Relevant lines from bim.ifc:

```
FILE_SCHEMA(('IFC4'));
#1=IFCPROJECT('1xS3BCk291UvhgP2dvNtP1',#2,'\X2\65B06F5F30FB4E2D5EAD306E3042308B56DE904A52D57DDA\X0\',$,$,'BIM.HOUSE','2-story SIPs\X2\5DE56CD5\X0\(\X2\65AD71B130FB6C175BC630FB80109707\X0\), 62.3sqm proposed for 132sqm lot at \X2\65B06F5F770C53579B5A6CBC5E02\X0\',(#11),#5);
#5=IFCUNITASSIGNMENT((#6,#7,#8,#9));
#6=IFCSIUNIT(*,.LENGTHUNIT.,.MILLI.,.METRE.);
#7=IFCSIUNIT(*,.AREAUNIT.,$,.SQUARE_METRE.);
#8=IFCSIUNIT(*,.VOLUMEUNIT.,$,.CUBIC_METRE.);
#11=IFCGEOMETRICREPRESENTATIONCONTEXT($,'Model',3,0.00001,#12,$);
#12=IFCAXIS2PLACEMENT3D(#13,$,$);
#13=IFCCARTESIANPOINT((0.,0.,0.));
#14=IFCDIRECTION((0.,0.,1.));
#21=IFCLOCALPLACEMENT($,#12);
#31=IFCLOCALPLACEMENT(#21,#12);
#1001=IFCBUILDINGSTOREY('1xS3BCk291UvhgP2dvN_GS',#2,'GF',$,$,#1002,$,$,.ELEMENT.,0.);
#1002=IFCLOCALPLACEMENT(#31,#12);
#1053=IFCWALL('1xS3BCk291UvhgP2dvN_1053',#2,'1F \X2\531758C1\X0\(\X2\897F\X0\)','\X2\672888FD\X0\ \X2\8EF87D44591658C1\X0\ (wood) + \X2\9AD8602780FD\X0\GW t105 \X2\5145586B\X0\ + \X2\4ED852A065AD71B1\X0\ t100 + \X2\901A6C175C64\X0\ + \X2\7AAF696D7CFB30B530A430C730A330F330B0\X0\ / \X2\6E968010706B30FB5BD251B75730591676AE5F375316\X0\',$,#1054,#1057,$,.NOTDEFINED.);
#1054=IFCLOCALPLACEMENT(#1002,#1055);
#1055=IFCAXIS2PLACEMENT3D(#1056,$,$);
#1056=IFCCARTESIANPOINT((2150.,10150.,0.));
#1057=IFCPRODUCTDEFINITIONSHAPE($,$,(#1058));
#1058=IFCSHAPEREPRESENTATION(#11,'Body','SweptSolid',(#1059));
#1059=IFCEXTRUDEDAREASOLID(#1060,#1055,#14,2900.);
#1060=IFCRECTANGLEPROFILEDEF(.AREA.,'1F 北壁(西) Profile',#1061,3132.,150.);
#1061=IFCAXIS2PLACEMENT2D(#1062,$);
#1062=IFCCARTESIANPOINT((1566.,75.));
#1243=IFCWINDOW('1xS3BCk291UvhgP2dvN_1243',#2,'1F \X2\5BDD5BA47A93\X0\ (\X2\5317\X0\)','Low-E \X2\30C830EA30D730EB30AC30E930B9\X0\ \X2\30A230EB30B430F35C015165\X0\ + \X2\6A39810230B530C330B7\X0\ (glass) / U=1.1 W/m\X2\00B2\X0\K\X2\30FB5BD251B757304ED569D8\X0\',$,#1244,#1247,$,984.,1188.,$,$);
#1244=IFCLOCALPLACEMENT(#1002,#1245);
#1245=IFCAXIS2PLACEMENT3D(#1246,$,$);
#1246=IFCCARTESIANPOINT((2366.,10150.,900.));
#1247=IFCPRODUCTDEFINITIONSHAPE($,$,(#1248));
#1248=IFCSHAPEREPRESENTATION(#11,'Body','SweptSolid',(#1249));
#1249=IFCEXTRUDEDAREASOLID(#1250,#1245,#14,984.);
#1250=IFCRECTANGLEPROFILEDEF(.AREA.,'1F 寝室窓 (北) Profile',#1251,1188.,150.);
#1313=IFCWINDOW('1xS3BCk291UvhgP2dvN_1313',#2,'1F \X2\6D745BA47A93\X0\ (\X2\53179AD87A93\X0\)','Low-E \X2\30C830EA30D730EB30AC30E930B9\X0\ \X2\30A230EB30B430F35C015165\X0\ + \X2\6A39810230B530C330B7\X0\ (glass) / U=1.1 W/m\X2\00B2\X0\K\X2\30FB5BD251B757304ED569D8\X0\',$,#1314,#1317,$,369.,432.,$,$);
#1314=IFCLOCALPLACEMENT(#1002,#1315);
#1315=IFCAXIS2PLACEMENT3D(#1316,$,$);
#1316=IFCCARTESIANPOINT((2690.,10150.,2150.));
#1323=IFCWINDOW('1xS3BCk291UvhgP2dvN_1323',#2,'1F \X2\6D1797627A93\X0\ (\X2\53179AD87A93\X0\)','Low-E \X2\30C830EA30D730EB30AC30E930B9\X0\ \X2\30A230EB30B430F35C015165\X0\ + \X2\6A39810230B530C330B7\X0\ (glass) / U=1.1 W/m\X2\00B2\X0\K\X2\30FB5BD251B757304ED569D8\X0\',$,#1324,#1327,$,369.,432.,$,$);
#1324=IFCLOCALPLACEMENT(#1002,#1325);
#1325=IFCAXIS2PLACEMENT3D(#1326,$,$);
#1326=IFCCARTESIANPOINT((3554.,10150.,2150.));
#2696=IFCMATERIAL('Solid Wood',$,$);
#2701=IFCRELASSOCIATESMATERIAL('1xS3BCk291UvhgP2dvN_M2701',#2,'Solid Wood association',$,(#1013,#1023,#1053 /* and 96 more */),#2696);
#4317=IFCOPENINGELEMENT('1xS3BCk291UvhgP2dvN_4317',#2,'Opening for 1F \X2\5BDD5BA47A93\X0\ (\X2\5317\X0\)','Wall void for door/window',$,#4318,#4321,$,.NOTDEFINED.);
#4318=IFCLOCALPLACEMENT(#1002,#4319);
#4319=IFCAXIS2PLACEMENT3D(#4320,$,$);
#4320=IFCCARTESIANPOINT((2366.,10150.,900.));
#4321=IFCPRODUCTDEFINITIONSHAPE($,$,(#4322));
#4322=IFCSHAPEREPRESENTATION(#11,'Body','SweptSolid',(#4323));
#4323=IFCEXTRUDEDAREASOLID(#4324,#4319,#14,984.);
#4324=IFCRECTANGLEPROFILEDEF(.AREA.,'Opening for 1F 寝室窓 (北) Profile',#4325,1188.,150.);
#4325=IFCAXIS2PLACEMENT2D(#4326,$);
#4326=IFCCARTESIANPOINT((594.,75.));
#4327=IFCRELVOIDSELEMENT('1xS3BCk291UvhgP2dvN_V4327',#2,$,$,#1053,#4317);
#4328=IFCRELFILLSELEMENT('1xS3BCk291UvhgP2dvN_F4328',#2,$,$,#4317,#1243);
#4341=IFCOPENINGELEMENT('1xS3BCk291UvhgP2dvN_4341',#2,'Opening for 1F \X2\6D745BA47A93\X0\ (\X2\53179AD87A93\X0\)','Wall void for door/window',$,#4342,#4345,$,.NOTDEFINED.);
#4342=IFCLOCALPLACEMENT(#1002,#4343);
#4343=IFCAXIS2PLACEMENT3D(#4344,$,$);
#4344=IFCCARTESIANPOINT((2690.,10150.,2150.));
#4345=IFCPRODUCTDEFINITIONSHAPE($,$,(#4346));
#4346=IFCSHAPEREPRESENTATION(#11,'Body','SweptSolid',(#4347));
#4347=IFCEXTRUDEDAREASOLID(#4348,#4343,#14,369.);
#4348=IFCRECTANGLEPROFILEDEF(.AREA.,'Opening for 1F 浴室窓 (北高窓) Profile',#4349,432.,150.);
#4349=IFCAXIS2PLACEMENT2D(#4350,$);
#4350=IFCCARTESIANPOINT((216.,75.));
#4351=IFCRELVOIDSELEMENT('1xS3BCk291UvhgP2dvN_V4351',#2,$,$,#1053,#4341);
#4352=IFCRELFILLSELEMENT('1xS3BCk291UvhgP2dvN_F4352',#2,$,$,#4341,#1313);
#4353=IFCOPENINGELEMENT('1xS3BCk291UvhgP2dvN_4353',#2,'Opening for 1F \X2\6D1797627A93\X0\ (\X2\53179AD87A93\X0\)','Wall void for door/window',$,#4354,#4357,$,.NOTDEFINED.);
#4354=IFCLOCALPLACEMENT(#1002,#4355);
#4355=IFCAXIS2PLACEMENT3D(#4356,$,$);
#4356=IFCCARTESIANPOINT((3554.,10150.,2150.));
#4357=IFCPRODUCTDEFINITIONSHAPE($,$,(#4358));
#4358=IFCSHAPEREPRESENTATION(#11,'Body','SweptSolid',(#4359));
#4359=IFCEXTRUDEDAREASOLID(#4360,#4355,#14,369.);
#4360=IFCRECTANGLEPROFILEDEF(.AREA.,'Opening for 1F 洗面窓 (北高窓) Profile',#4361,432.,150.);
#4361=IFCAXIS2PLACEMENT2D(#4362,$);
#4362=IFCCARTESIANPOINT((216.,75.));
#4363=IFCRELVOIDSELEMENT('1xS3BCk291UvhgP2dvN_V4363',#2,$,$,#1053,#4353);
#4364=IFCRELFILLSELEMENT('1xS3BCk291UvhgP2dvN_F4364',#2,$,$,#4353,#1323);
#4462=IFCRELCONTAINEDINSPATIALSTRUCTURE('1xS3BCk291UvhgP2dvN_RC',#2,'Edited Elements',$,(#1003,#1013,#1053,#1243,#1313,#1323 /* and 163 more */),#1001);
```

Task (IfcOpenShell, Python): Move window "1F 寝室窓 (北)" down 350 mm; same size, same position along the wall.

```python
import numpy as np
import ifcopenshell
import ifcopenshell.api.geometry
import ifcopenshell.util.placement
import ifcopenshell.util.unit

model = ifcopenshell.open("bim.ifc")
unit_scale = ifcopenshell.util.unit.calculate_unit_scale(model)

window = model.by_guid("1xS3BCk291UvhgP2dvN_1243")
opening = window.FillsVoids[0].RelatingOpeningElement
dz = -350.0

shift = np.array([0.0, 0.0, dz])
# The window is not placed relative to its opening, so move both.
for product in (opening, window):
    matrix = ifcopenshell.util.placement.get_local_placement(product.ObjectPlacement)
    matrix[:3, 3] += shift
    ifcopenshell.api.geometry.edit_object_placement(model, product=product, matrix=matrix, is_si=False)

print(f"moved by {dz * unit_scale:+.3f} m")

model.write("bim_rev.ifc")
```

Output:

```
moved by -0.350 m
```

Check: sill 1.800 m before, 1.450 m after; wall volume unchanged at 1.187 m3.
